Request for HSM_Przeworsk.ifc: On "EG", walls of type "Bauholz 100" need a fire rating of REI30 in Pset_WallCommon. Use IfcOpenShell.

First a look at what the model holds.

```python
import ifcopenshell
import ifcopenshell.util.element

model = ifcopenshell.open("HSM_Przeworsk.ifc")
print(model.schema)
storey = next(s for s in model.by_type("IfcBuildingStorey") if s.Name == "EG")
walls = [e for e in ifcopenshell.util.element.get_decomposition(storey) if e.is_a("IfcWall")]
seen = {}
for e in walls:
    element_type = ifcopenshell.util.element.get_type(e)
    key = (element_type.Name if element_type != e and element_type else None, ifcopenshell.util.element.get_pset(e, "Pset_WallCommon", "FireRating"))
    seen[key] = seen.get(key, 0) + 1
for (name, value), count in sorted(seen.items(), key=str):
    print(count, "x", name, "|", value)
```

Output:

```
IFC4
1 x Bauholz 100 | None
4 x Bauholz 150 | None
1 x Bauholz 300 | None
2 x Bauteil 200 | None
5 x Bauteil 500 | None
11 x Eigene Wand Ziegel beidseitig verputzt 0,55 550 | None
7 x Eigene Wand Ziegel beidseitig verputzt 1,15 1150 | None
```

```python
import ifcopenshell
import ifcopenshell.api.pset
import ifcopenshell.util.element

model = ifcopenshell.open("HSM_Przeworsk.ifc")

storey = next(s for s in model.by_type("IfcBuildingStorey") if s.Name == "EG")
walls = [e for e in ifcopenshell.util.element.get_decomposition(storey) if e.is_a("IfcWall")]

count = 0
for e in walls:
    element_type = ifcopenshell.util.element.get_type(e)
    if element_type in (None, e) or element_type.Name != "Bauholz 100":
        continue
    # add_pset returns the element's existing set when there is one.
    pset = ifcopenshell.api.pset.add_pset(model, product=e, name="Pset_WallCommon")
    ifcopenshell.api.pset.edit_pset(model, pset=pset, properties={"FireRating": "REI30"})
    count += 1

print(count, "walls updated")

model.write("HSM_Przeworsk_updated.ifc")
```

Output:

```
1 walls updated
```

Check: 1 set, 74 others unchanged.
